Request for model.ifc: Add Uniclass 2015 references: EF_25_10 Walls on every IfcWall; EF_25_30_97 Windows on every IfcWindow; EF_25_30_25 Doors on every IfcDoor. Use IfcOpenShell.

First a look at what the model holds.

```python
import ifcopenshell

model = ifcopenshell.open("model.ifc")
print(model.schema)
print("classifications:", [c.Name for c in model.by_type("IfcClassification")])
for ifc_class in ("IfcDoor", "IfcRoof", "IfcStair", "IfcWall", "IfcWindow"):
    print(ifc_class, len(model.by_type(ifc_class)))
```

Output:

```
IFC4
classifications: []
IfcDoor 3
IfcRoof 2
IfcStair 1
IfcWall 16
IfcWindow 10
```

```python
import ifcopenshell
import ifcopenshell.api.classification

model = ifcopenshell.open("model.ifc")

system = ifcopenshell.api.classification.add_classification(model, classification="Uniclass 2015")

codes = {
    "IfcWall": ("EF_25_10", "Walls"),
    "IfcWindow": ("EF_25_30_97", "Windows"),
    "IfcDoor": ("EF_25_30_25", "Doors"),
}
for ifc_class, (code, name) in codes.items():
    products = model.by_type(ifc_class)
    ifcopenshell.api.classification.add_reference(
        model, products=products, classification=system, identification=code, name=name
    )
    print(code, len(products))

model.write("model_updated.ifc")
```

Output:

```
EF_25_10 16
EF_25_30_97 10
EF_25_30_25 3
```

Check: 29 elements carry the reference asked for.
